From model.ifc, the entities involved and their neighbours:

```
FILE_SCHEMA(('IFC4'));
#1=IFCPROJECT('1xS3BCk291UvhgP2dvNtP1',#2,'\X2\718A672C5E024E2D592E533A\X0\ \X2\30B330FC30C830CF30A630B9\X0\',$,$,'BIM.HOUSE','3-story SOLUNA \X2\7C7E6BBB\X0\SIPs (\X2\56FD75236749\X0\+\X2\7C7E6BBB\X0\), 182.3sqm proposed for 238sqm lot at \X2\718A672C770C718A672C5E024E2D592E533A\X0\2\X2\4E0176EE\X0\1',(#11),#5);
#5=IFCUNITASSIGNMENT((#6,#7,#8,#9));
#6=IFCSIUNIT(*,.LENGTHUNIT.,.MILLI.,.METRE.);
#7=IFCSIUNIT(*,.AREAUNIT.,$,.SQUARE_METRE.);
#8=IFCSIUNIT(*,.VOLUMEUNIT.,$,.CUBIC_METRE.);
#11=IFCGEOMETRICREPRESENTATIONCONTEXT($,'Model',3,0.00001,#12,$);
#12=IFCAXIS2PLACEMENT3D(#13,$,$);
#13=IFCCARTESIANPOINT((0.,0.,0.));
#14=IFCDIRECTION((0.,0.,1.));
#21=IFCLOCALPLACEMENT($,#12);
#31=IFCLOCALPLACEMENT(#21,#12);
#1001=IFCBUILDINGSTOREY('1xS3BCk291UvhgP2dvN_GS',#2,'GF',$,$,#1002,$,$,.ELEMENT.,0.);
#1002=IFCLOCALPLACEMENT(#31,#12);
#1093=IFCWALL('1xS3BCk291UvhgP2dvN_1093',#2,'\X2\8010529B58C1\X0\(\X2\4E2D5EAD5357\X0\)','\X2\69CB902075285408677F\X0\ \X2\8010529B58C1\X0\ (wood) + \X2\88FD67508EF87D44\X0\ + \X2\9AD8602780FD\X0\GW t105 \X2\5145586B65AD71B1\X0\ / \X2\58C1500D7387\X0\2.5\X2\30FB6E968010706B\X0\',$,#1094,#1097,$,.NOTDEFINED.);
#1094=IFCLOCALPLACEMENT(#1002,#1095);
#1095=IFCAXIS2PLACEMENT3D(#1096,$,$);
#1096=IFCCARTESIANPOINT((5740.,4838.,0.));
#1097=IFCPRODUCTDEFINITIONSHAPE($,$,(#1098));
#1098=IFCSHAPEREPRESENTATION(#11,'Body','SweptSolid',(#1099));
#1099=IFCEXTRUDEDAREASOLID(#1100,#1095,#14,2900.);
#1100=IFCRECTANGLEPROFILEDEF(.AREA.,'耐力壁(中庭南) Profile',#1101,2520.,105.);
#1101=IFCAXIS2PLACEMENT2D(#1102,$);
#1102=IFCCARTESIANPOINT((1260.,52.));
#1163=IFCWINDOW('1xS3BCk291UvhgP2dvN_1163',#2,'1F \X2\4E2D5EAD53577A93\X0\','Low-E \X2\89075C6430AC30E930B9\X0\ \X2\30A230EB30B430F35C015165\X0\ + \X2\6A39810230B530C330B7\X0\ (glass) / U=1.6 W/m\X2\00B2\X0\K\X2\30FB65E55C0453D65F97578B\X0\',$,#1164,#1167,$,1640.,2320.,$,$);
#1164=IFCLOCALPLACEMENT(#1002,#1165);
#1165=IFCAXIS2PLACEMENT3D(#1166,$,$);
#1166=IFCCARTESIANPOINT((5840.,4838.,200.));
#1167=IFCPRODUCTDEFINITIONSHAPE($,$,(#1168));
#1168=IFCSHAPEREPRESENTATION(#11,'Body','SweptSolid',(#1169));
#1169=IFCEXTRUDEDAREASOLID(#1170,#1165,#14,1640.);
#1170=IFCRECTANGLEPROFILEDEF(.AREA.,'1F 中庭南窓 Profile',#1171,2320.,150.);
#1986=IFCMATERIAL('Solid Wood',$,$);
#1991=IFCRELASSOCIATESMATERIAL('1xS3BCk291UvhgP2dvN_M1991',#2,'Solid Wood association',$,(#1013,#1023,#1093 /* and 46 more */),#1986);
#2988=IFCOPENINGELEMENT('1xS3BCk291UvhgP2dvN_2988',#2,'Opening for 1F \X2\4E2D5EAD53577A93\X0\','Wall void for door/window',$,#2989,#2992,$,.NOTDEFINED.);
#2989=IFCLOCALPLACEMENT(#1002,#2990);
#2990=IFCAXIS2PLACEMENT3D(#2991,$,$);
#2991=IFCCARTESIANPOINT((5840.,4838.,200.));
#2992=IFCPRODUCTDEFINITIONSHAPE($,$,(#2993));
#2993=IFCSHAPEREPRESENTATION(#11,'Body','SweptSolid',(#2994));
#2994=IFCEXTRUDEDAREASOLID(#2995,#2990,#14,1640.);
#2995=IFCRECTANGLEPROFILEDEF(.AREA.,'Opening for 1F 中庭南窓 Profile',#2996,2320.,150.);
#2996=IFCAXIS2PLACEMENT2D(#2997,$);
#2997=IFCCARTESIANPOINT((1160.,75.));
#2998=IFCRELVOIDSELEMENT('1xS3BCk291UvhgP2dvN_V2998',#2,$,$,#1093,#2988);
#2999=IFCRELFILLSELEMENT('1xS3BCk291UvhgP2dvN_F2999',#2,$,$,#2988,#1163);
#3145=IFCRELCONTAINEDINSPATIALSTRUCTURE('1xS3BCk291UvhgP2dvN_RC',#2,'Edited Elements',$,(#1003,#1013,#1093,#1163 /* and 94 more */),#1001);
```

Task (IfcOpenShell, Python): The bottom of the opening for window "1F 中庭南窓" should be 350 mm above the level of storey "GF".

```python
import numpy as np
import ifcopenshell
import ifcopenshell.api.geometry
import ifcopenshell.geom
import ifcopenshell.util.element
import ifcopenshell.util.placement
import ifcopenshell.util.shape
import ifcopenshell.util.unit

model = ifcopenshell.open("model.ifc")
unit_scale = ifcopenshell.util.unit.calculate_unit_scale(model)

window = model.by_guid("1xS3BCk291UvhgP2dvN_1163")
opening = window.FillsVoids[0].RelatingOpeningElement
storey = ifcopenshell.util.element.get_container(window, ifc_class="IfcBuildingStorey")
level = ifcopenshell.util.placement.get_local_placement(storey.ObjectPlacement)[2, 3]

# The opening's origin need not be at the sill, so measure its lowest point.
shape = ifcopenshell.geom.create_shape(ifcopenshell.geom.settings(), opening)
bottom = ifcopenshell.util.shape.get_shape_bottom_elevation(shape, shape.geometry) / unit_scale
dz = level + 0.35 / unit_scale - bottom

shift = np.array([0.0, 0.0, dz])
# The window is not placed relative to its opening, so move both.
for product in (opening, window):
    matrix = ifcopenshell.util.placement.get_local_placement(product.ObjectPlacement)
    matrix[:3, 3] += shift
    ifcopenshell.api.geometry.edit_object_placement(model, product=product, matrix=matrix, is_si=False)

print(f"moved by {dz * unit_scale:+.3f} m")

model.write("model_updated.ifc")
```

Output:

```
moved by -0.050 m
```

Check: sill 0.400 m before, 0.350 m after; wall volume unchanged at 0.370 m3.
